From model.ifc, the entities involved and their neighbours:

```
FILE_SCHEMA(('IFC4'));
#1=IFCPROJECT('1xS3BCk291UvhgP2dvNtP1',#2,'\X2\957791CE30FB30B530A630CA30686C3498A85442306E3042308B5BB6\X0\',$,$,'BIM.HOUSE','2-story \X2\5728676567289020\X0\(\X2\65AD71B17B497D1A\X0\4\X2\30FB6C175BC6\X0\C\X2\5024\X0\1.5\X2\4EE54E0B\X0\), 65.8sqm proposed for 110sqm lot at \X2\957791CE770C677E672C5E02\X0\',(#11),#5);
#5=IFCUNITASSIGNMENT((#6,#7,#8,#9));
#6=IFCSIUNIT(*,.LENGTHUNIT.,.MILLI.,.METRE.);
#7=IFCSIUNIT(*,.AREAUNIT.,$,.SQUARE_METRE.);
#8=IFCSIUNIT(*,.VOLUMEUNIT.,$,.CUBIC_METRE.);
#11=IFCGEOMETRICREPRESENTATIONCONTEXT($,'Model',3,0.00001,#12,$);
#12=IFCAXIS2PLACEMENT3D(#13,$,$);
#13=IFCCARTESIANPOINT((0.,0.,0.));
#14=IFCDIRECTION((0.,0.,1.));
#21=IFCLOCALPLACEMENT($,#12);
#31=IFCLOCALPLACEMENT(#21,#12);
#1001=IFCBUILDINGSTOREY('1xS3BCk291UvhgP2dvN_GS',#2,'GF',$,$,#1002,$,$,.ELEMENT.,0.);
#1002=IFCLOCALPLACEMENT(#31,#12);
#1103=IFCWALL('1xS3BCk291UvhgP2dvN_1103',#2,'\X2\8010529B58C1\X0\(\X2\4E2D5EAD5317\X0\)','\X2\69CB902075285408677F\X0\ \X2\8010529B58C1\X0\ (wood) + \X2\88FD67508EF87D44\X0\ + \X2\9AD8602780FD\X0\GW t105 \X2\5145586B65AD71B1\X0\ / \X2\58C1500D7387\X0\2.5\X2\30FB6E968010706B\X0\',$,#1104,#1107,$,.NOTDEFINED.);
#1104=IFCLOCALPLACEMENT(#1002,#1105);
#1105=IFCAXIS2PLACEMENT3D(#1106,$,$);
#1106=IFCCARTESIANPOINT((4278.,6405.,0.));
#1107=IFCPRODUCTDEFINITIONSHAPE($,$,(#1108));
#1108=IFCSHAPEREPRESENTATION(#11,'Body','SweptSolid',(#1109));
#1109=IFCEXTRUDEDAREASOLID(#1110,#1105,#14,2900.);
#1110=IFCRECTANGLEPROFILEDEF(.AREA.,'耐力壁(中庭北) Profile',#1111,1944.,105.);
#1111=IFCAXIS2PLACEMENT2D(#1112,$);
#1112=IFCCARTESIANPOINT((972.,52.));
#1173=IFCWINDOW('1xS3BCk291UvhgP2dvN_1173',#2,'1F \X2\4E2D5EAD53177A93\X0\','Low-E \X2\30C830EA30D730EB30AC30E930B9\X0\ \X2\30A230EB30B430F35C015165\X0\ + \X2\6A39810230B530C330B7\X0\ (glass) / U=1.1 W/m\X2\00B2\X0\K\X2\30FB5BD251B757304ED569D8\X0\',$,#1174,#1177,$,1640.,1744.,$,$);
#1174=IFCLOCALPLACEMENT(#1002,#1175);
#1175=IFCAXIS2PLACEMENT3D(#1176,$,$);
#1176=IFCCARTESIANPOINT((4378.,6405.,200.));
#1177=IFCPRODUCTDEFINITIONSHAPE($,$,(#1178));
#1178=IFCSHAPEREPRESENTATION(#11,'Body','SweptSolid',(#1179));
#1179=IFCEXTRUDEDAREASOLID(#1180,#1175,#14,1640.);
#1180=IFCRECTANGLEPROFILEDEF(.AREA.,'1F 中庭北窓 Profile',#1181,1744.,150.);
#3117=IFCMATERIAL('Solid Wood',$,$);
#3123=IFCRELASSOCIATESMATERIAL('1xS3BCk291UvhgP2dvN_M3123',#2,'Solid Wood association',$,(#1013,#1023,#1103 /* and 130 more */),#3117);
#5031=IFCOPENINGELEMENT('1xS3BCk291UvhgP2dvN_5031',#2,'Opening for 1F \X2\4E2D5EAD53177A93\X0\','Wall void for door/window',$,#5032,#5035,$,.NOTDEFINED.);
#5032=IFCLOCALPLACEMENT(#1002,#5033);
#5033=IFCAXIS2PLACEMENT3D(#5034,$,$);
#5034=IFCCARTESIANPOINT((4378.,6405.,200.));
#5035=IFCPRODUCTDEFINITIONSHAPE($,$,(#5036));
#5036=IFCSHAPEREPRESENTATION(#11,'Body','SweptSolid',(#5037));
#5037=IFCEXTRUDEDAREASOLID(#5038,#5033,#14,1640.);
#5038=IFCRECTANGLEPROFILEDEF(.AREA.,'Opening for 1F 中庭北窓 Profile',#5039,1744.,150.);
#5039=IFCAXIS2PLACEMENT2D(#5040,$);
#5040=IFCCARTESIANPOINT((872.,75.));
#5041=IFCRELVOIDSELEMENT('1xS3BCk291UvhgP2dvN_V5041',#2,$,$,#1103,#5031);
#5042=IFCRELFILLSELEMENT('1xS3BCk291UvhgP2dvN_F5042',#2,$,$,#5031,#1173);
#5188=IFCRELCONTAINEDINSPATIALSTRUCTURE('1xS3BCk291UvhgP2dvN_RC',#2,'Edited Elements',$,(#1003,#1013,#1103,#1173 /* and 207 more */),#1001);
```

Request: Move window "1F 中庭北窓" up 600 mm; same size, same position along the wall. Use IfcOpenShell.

```python
import numpy as np
import ifcopenshell
import ifcopenshell.api.geometry
import ifcopenshell.util.placement
import ifcopenshell.util.unit

model = ifcopenshell.open("model.ifc")
unit_scale = ifcopenshell.util.unit.calculate_unit_scale(model)

window = model.by_id(1173)
opening = window.FillsVoids[0].RelatingOpeningElement
dz = 0.6 / unit_scale

shift = np.array([0.0, 0.0, dz])
# The window is not placed relative to its opening, so move both.
for product in (opening, window):
    matrix = ifcopenshell.util.placement.get_local_placement(product.ObjectPlacement)
    matrix[:3, 3] += shift
    ifcopenshell.api.geometry.edit_object_placement(model, product=product, matrix=matrix, is_si=False)

print(f"moved by {dz * unit_scale:+.3f} m")

model.write("model_v2.ifc")
```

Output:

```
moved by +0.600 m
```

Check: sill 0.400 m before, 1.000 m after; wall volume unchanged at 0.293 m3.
